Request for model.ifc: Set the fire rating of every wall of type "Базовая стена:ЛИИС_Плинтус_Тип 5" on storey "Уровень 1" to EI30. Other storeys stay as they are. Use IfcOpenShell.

First a look at what the model holds.

```python
import ifcopenshell
import ifcopenshell.util.element

model = ifcopenshell.open("model.ifc")
print(model.schema)
storey = next(s for s in model.by_type("IfcBuildingStorey") if s.Name == "Уровень 1")
walls = [e for e in ifcopenshell.util.element.get_decomposition(storey) if e.is_a("IfcWall")]
seen = {}
for e in walls:
    element_type = ifcopenshell.util.element.get_type(e)
    key = (element_type.Name if element_type != e and element_type else None, ifcopenshell.util.element.get_pset(e, "Pset_WallCommon", "FireRating"))
    seen[key] = seen.get(key, 0) + 1
for (name, value), count in sorted(seen.items(), key=str):
    print(count, "x", name, "|", value)
```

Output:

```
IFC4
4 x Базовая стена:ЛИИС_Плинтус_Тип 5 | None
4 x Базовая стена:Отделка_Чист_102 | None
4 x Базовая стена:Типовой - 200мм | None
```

```python
import ifcopenshell
import ifcopenshell.api.pset
import ifcopenshell.util.element

model = ifcopenshell.open("model.ifc")

storey = next(s for s in model.by_type("IfcBuildingStorey") if s.Name == "Уровень 1")
walls = [e for e in ifcopenshell.util.element.get_decomposition(storey) if e.is_a("IfcWall")]

count = 0
for e in walls:
    element_type = ifcopenshell.util.element.get_type(e)
    if element_type in (None, e) or element_type.Name != "Базовая стена:ЛИИС_Плинтус_Тип 5":
        continue
    # add_pset returns the element's existing set when there is one.
    pset = ifcopenshell.api.pset.add_pset(model, product=e, name="Pset_WallCommon")
    ifcopenshell.api.pset.edit_pset(model, pset=pset, properties={"FireRating": "EI30"})
    count += 1

print(count, "walls updated")

model.write("model_edited.ifc")
```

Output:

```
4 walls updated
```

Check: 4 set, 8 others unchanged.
